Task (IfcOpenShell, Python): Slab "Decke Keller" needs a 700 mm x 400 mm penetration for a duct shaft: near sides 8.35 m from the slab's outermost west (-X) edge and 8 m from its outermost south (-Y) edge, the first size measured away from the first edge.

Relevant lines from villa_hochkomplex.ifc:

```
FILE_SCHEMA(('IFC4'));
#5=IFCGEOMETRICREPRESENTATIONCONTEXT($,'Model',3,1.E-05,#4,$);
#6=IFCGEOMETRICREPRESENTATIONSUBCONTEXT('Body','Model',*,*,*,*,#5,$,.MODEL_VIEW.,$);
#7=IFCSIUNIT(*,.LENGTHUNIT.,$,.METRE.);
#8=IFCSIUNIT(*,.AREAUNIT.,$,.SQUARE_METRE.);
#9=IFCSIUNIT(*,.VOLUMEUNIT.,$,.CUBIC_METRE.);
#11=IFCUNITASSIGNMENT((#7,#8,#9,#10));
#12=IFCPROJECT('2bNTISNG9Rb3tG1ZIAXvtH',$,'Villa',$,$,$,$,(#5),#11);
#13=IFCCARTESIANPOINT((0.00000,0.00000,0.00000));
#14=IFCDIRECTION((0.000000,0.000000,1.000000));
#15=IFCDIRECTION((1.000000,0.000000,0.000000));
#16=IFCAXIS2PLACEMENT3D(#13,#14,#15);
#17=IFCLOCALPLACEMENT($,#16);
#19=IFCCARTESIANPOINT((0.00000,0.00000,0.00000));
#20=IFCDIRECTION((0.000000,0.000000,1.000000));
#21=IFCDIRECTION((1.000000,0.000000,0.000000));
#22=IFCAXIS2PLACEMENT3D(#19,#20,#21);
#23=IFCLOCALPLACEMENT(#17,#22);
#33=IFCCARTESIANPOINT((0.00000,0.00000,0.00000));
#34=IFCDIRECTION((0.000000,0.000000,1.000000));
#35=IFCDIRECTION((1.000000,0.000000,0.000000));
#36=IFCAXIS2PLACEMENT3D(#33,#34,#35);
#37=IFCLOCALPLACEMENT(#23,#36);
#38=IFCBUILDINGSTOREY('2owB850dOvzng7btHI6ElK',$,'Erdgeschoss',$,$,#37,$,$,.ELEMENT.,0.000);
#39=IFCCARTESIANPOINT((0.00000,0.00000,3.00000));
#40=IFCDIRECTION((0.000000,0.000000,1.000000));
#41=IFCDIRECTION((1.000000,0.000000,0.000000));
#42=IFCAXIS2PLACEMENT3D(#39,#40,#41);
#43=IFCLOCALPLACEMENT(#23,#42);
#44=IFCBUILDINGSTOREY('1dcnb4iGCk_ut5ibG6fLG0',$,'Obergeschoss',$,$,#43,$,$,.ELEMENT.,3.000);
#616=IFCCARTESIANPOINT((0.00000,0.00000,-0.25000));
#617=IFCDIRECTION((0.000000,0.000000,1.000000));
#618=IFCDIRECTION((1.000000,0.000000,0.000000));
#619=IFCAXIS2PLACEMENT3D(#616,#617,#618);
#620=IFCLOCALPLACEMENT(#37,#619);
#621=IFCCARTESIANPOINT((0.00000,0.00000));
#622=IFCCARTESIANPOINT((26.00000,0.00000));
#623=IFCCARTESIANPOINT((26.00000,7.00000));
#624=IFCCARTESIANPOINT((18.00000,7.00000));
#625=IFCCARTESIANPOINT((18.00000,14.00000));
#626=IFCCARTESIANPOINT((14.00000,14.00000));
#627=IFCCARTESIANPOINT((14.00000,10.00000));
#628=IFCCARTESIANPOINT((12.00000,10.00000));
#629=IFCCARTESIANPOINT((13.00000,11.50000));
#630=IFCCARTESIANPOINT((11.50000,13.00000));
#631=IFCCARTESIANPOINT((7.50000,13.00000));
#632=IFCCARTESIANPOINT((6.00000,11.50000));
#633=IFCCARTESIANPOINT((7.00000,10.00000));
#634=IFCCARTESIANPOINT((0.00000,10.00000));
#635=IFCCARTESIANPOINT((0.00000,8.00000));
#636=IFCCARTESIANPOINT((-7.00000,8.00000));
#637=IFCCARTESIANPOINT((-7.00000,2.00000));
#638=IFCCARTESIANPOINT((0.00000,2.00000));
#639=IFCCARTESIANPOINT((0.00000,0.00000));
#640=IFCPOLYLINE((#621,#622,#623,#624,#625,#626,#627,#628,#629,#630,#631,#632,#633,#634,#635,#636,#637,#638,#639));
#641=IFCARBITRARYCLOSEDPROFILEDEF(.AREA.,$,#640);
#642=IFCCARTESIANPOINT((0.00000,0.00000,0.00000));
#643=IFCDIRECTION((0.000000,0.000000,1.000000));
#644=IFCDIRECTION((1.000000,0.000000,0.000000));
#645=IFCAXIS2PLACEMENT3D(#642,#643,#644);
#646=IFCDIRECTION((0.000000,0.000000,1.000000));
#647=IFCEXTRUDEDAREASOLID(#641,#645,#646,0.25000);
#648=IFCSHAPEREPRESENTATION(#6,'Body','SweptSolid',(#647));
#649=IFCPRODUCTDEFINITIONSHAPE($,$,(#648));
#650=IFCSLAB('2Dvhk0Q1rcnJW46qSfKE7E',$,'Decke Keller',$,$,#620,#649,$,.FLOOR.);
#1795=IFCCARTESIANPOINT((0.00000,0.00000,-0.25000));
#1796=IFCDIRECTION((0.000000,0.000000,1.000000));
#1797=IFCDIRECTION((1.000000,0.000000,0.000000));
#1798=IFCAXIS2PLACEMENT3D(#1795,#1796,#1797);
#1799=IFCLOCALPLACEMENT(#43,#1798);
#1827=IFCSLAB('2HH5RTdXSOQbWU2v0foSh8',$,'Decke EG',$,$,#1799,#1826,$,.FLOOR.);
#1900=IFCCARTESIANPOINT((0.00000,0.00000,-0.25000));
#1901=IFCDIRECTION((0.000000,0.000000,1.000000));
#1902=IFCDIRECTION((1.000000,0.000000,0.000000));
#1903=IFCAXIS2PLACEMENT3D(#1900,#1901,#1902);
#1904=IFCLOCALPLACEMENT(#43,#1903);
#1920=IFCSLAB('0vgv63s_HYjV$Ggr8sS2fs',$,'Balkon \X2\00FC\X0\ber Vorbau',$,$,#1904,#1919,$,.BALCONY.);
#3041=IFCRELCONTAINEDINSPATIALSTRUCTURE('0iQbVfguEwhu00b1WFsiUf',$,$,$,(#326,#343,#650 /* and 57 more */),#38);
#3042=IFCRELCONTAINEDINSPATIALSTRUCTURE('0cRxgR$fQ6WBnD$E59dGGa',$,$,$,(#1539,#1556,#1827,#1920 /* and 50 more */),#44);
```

```python
import numpy as np
import ifcopenshell
import ifcopenshell.api.feature
import ifcopenshell.api.geometry
import ifcopenshell.api.root
import ifcopenshell.geom
import ifcopenshell.util.placement
import ifcopenshell.util.representation
import ifcopenshell.util.shape
import ifcopenshell.util.unit

model = ifcopenshell.open("villa_hochkomplex.ifc")
unit_scale = ifcopenshell.util.unit.calculate_unit_scale(model)
settings = ifcopenshell.geom.settings()


def volume(element):
    """Net volume in cubic metres, openings subtracted."""
    shape = ifcopenshell.geom.create_shape(settings, element)
    return ifcopenshell.util.shape.get_volume(shape.geometry)


slab = model.by_guid("2Dvhk0Q1rcnJW46qSfKE7E")
before = volume(slab)

# Extent in the slab's own axes, in metres. The edges named are its -X and -Y sides.
slab_shape = ifcopenshell.geom.create_shape(settings, slab)
vertices = ifcopenshell.util.shape.get_vertices(slab_shape.geometry)
x_min, y_min, bottom = vertices.min(axis=0)
top = vertices[:, 2].max()

opening = ifcopenshell.api.root.create_entity(model, ifc_class="IfcOpeningElement", name="Duct shaft opening", predefined_type="OPENING")
context = ifcopenshell.util.representation.get_context(model, "Model", "Body", "MODEL_VIEW")
width, depth = 0.7, 0.4
outline = [(0.0, 0.0), (width, 0.0), (width, depth), (0.0, depth), (0.0, 0.0)]
# Overshoot both faces by 50 mm so the cut is clean.
shape = ifcopenshell.api.geometry.add_slab_representation(
    model, context=context, depth=top - bottom + 0.1, polyline=outline
)
ifcopenshell.api.geometry.assign_representation(model, product=opening, representation=shape)

matrix = ifcopenshell.util.placement.get_local_placement(slab.ObjectPlacement)
matrix[:, 3] = matrix @ np.append(np.array([x_min + 8.35, y_min + 8, bottom - 0.05]) / unit_scale, 1.0)
ifcopenshell.api.geometry.edit_object_placement(model, product=opening, matrix=matrix, is_si=False)
ifcopenshell.api.feature.add_feature(model, feature=opening, element=slab)

after = volume(slab)

print(f"slab volume {before:.3f} -> {after:.3f} m3")

model.write("villa_hochkomplex_v2.ifc")
```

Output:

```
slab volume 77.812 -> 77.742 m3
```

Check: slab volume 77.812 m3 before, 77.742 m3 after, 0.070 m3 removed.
